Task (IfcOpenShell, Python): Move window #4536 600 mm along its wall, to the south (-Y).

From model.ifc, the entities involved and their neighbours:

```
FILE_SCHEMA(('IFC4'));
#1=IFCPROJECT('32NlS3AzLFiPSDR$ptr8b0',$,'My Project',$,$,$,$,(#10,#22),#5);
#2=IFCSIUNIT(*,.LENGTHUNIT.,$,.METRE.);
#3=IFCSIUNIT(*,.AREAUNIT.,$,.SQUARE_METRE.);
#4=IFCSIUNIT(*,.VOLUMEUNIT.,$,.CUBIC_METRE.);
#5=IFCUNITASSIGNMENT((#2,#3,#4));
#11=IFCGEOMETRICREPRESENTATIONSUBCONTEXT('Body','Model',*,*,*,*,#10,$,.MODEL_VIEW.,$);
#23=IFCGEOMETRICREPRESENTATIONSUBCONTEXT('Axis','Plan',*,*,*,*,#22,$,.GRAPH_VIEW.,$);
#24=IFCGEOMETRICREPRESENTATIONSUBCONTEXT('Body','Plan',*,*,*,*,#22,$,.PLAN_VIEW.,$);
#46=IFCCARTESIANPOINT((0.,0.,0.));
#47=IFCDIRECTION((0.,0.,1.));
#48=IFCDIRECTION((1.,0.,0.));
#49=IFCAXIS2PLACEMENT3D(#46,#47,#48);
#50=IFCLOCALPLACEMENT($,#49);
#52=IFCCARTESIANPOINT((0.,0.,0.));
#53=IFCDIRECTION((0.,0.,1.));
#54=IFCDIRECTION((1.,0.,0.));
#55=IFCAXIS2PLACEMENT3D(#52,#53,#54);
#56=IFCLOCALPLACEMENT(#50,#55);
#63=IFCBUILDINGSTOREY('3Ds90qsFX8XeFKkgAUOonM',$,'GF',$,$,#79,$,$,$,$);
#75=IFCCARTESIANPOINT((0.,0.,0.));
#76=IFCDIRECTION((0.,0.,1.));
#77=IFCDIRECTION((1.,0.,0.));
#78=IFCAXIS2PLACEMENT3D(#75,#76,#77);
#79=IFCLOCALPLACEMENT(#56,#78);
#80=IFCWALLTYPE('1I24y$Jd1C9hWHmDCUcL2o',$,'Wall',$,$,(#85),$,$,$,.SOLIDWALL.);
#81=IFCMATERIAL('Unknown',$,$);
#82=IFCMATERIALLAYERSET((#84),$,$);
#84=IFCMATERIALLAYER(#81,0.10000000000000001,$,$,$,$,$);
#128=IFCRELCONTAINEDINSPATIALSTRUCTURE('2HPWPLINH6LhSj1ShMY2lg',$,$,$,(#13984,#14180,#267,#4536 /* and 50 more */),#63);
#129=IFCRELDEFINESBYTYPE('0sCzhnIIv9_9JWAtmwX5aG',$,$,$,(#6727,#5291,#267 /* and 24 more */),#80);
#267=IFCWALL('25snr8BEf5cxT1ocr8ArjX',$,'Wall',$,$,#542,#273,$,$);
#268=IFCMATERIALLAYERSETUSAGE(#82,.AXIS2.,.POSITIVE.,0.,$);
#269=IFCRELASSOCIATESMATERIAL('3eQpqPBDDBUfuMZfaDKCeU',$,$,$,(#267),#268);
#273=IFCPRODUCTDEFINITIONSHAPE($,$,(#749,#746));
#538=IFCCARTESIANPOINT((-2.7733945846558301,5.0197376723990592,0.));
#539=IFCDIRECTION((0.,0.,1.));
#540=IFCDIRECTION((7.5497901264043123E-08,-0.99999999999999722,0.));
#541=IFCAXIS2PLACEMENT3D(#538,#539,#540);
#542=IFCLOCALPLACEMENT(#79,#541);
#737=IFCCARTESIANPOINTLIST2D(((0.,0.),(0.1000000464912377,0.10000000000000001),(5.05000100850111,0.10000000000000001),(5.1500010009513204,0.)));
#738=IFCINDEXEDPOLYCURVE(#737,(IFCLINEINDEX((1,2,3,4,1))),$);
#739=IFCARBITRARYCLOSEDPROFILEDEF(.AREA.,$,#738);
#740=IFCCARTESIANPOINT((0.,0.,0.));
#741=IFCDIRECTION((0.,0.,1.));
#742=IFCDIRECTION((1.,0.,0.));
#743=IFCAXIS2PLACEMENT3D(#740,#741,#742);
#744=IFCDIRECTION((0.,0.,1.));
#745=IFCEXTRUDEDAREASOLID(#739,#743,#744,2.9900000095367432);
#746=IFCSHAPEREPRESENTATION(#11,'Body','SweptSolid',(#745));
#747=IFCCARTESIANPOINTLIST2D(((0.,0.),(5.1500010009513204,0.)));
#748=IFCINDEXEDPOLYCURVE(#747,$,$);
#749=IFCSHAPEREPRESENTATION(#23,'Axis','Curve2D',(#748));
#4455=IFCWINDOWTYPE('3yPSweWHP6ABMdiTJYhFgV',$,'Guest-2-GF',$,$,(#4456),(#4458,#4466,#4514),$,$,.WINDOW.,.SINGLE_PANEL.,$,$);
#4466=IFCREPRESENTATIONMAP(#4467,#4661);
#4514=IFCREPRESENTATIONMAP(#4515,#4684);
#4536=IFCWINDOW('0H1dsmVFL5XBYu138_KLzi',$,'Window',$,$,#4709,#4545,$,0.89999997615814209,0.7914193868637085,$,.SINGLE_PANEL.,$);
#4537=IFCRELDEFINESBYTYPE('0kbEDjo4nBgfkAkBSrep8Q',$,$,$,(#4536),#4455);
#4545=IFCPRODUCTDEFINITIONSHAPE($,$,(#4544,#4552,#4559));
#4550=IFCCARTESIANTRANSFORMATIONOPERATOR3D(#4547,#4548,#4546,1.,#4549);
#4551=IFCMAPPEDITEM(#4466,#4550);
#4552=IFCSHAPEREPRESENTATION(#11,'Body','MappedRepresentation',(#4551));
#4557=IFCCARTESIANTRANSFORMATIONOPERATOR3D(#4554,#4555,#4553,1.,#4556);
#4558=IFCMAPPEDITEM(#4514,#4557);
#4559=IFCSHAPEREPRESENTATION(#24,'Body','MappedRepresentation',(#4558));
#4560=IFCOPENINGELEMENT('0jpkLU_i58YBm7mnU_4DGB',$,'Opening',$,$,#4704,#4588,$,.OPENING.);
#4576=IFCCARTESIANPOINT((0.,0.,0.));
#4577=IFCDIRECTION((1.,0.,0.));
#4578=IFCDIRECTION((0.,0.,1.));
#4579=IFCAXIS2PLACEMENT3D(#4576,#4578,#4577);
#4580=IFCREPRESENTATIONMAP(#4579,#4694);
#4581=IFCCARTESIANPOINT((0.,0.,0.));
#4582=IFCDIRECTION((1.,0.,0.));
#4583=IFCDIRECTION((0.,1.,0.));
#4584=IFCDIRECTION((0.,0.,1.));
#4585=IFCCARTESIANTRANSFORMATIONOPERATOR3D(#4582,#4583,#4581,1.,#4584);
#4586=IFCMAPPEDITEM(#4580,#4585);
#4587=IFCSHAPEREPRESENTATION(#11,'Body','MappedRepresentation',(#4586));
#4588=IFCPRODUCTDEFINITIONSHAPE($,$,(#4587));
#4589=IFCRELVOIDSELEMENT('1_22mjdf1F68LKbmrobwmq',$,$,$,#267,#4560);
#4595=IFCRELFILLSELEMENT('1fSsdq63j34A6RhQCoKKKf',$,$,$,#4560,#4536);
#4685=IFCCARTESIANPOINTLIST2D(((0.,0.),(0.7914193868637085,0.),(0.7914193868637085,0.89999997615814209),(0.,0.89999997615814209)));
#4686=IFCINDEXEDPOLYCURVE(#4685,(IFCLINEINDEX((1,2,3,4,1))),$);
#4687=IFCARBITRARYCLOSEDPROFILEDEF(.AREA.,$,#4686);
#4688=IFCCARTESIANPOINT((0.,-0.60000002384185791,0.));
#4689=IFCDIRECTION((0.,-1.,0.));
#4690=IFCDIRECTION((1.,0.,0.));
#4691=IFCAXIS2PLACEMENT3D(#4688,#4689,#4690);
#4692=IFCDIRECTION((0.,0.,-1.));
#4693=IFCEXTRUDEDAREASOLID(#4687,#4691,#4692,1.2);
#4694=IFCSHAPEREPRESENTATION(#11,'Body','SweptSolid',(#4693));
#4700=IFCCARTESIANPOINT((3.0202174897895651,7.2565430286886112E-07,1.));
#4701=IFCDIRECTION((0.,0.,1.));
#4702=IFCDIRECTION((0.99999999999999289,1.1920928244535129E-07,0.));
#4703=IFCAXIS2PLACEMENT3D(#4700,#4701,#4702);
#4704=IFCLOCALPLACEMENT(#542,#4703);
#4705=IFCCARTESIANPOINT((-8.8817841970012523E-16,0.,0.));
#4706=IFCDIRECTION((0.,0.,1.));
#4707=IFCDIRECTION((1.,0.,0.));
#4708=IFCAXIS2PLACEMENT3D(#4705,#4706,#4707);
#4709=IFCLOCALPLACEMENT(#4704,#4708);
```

```python
import ifcopenshell
import ifcopenshell.api.geometry
import ifcopenshell.util.placement

model = ifcopenshell.open("model.ifc")

window = model.by_guid("0H1dsmVFL5XBYu138_KLzi")
opening = window.FillsVoids[0].RelatingOpeningElement
wall = opening.VoidsElements[0].RelatingBuildingElement

wall_matrix = ifcopenshell.util.placement.get_local_placement(wall.ObjectPlacement)
shift = wall_matrix[:3, 0] * 0.6
before = ifcopenshell.util.placement.get_local_placement(window.ObjectPlacement)[:3, 3].copy()

# The window is placed relative to its opening, so it follows when the opening moves.
matrix = ifcopenshell.util.placement.get_local_placement(opening.ObjectPlacement)
matrix[:3, 3] += shift
ifcopenshell.api.geometry.edit_object_placement(
    model, product=opening, matrix=matrix, is_si=False, should_transform_children=True
)

after = ifcopenshell.util.placement.get_local_placement(window.ObjectPlacement)[:3, 3]
print("window moved by", (after - before).round(3) + 0.0)

model.write("model-out.ifc")
```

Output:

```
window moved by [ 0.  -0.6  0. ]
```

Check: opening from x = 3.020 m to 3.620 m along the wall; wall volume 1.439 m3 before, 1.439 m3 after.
